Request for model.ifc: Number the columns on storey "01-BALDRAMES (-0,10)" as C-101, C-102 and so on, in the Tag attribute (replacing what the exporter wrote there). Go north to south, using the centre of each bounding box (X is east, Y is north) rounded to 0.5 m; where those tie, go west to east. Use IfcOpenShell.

First a look at what the model holds.

```python
import ifcopenshell
import ifcopenshell.util.element
import ifcopenshell.util.placement

model = ifcopenshell.open("model.ifc")
print(model.schema)
storey = next(s for s in model.by_type("IfcBuildingStorey") if s.Name == "01-BALDRAMES (-0,10)")
columns = [e for e in ifcopenshell.util.element.get_decomposition(storey) if e.is_a("IfcColumn")]
for e in sorted(columns, key=lambda e: e.id()):
    origin = ifcopenshell.util.placement.get_local_placement(e.ObjectPlacement)[:3, 3]
    print(e.id(), e.Tag, e.Name, origin.round(2) + 0.0, sep=" | ")
```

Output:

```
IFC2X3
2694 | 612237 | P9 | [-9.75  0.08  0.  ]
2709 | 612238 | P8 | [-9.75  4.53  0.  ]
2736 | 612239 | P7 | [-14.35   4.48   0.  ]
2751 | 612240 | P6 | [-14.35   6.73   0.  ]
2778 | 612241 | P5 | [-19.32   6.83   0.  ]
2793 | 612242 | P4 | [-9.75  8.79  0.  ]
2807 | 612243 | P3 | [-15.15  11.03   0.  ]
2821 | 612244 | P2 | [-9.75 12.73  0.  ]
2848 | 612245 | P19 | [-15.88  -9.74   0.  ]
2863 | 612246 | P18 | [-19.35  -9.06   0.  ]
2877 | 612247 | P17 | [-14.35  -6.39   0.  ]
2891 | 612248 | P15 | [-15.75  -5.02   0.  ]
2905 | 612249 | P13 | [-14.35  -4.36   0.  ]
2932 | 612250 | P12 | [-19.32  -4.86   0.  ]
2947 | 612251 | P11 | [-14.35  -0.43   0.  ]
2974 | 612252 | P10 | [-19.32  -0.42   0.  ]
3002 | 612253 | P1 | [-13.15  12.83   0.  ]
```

```python
import ifcopenshell
import ifcopenshell.geom
import ifcopenshell.util.element
import ifcopenshell.util.shape

model = ifcopenshell.open("model.ifc")
settings = ifcopenshell.geom.settings()
settings.set("use-world-coords", True)


def centre(element):
    shape = ifcopenshell.geom.create_shape(settings, element)
    return ifcopenshell.util.shape.get_bbox_centroid(shape.geometry)


storey = next(s for s in model.by_type("IfcBuildingStorey") if s.Name == "01-BALDRAMES (-0,10)")
columns = [e for e in ifcopenshell.util.element.get_decomposition(storey) if e.is_a("IfcColumn")]

# Insertion points can sit at a corner or the storey origin, so sort by the geometry (in metres).
centres = {e: centre(e) for e in columns}
columns.sort(key=lambda e: (-round(centres[e][1] / 0.5), centres[e][0]))

for i, e in enumerate(columns, start=1):
    number = f"C-1{i:02d}"
    e.Tag = number
    print(e.id(), number)

model.write("model_updated.ifc")
```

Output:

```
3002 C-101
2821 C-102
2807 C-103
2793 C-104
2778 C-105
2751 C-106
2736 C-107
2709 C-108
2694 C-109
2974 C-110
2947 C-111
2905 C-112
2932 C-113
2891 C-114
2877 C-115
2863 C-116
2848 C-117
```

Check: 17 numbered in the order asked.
